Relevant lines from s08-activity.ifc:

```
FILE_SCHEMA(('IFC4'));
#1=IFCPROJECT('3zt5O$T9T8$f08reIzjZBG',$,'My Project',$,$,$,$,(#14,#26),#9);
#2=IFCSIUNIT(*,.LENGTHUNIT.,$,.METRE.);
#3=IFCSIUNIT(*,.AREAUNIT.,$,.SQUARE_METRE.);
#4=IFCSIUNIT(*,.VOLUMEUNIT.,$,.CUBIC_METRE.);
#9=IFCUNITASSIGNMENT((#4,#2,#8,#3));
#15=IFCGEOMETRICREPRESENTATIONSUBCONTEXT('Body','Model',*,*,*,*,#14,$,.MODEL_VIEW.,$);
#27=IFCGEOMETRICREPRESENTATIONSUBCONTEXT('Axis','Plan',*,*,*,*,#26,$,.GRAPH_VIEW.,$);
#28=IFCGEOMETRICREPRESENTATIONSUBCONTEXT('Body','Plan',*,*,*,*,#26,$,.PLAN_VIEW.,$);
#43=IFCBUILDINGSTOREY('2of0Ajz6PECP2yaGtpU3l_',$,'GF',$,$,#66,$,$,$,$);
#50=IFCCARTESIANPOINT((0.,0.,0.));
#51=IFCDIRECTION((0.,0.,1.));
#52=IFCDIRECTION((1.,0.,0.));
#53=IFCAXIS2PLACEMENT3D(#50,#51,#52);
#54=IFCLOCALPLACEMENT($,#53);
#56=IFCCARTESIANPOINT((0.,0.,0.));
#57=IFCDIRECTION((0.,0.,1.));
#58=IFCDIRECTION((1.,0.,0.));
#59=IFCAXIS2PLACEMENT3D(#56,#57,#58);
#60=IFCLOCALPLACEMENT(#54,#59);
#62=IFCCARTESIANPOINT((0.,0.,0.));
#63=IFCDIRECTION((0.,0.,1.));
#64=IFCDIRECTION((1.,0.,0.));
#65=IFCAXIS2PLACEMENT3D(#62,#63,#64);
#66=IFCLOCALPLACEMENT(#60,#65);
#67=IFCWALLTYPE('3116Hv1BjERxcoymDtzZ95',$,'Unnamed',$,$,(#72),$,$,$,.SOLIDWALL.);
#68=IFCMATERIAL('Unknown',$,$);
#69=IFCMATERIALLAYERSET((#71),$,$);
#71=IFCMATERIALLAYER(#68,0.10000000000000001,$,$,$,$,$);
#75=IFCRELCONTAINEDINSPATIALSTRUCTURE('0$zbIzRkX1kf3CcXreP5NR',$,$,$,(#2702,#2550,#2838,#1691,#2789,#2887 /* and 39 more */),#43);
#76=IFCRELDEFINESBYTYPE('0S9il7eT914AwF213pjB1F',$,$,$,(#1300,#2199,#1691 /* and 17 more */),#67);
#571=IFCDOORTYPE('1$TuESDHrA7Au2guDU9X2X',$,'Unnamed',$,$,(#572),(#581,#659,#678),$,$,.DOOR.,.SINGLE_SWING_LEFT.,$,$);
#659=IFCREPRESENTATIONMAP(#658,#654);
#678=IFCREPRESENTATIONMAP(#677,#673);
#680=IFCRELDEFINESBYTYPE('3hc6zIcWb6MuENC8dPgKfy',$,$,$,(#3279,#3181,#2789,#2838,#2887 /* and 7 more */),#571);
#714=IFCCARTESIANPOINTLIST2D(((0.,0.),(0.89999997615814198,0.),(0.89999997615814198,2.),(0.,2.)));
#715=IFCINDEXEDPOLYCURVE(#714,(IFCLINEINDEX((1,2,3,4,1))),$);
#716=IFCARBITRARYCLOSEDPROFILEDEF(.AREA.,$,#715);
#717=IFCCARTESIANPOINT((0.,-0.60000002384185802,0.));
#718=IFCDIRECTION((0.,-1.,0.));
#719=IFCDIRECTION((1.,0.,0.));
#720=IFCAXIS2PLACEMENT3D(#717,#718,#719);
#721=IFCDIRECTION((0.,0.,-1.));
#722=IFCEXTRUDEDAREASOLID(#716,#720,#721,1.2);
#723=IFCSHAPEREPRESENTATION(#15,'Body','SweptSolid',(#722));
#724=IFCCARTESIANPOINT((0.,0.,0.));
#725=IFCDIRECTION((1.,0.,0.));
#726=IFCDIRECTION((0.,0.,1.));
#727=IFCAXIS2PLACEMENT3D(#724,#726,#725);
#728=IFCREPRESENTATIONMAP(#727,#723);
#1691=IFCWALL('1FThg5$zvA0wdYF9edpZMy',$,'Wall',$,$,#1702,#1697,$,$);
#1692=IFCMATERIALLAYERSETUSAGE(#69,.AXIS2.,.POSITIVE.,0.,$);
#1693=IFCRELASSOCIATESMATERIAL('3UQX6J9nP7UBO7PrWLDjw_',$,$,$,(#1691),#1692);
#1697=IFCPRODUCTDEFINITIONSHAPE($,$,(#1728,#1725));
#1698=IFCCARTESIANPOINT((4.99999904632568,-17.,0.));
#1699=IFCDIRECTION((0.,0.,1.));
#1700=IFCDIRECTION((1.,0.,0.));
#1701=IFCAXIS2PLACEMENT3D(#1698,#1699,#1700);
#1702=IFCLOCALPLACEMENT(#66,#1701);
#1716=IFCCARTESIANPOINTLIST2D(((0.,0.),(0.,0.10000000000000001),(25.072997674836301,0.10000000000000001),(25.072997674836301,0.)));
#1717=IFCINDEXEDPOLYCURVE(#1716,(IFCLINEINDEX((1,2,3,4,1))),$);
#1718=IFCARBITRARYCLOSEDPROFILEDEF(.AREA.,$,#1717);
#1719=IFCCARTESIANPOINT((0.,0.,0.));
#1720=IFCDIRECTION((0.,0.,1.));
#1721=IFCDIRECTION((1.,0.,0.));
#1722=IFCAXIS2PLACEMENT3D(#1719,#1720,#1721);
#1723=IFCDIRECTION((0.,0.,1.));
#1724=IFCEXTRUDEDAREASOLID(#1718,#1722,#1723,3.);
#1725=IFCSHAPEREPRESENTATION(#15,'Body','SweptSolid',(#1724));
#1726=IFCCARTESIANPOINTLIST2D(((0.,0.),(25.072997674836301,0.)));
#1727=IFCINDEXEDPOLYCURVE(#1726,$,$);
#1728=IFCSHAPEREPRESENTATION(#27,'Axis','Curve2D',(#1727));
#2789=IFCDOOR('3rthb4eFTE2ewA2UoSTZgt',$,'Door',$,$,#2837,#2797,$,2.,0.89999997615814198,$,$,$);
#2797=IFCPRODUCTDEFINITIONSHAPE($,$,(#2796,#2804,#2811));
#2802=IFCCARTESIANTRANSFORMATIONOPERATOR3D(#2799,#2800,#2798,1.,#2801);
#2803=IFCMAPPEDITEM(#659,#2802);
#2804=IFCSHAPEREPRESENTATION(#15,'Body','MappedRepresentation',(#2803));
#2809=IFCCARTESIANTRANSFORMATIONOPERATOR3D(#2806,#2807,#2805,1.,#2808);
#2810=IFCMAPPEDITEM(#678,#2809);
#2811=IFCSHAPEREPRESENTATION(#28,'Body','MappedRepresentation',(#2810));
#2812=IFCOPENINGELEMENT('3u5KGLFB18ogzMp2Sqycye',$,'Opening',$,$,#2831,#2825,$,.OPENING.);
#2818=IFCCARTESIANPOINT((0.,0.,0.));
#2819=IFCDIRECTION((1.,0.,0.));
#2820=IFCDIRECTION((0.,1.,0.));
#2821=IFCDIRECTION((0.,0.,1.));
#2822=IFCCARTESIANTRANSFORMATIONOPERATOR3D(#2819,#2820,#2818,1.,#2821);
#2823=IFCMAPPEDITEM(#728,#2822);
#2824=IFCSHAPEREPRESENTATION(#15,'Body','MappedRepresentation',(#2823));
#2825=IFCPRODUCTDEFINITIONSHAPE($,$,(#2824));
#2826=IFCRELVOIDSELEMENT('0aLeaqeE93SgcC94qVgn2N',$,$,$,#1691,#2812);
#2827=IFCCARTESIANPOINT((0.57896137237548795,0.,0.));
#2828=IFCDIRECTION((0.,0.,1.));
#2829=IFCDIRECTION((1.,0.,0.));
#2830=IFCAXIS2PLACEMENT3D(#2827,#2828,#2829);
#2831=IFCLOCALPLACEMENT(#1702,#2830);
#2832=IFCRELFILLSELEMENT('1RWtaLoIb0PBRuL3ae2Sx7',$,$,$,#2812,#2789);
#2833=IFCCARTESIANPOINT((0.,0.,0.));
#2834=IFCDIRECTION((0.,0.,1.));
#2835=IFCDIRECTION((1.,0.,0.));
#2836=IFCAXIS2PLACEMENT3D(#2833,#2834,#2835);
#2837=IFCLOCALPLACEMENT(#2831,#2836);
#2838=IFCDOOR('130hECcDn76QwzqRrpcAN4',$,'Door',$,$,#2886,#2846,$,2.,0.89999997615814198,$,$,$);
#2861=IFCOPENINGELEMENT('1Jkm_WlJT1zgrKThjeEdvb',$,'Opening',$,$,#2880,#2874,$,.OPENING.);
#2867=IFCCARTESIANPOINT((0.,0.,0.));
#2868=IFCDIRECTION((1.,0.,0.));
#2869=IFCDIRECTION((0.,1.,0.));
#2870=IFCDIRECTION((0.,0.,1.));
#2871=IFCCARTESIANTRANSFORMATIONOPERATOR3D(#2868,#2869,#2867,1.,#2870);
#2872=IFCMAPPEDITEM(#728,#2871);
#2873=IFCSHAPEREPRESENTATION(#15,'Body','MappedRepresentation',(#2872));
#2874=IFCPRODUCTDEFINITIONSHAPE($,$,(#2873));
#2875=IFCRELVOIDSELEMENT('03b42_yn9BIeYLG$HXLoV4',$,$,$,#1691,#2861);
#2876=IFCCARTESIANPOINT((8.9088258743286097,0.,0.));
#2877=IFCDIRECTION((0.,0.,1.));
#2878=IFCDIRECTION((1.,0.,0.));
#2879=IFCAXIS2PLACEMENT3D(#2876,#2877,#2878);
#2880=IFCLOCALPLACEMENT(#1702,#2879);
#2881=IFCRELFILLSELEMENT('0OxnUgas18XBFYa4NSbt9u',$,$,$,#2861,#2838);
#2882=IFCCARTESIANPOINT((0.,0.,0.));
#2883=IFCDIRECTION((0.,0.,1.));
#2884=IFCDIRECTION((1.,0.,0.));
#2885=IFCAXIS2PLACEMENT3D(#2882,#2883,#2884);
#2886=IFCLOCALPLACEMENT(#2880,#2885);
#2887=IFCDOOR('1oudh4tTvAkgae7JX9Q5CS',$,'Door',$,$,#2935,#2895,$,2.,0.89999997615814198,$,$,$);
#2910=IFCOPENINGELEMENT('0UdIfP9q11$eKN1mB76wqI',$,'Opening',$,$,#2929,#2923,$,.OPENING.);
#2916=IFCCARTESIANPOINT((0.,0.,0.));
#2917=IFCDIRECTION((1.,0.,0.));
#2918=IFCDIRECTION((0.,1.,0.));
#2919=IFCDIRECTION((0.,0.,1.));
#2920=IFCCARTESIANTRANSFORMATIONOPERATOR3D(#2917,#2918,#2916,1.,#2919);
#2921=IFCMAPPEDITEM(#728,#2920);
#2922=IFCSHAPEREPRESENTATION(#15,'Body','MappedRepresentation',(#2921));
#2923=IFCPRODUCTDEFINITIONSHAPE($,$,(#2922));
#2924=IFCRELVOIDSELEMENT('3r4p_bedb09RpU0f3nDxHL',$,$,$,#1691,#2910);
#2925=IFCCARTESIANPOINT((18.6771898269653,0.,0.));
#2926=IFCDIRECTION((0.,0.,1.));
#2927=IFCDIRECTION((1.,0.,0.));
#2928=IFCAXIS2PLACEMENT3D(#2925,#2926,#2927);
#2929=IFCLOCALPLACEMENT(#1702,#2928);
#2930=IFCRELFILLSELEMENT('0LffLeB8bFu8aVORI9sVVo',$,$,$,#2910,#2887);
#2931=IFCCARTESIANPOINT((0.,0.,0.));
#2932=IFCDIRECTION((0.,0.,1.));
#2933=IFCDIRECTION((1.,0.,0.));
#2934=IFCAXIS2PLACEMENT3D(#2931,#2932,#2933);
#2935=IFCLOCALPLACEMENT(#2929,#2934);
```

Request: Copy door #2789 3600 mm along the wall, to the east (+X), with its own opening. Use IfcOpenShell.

```python
import ifcopenshell
import ifcopenshell.api.feature
import ifcopenshell.api.geometry
import ifcopenshell.api.root
import ifcopenshell.geom
import ifcopenshell.util.element
import ifcopenshell.util.placement
import ifcopenshell.util.shape
import ifcopenshell.util.unit

model = ifcopenshell.open("s08-activity.ifc")
unit_scale = ifcopenshell.util.unit.calculate_unit_scale(model)
settings = ifcopenshell.geom.settings()


def volume(element):
    """Net volume in cubic metres, openings subtracted."""
    shape = ifcopenshell.geom.create_shape(settings, element)
    return ifcopenshell.util.shape.get_volume(shape.geometry)


door = model.by_guid("3rthb4eFTE2ewA2UoSTZgt")
opening = door.FillsVoids[0].RelatingOpeningElement
wall = opening.VoidsElements[0].RelatingBuildingElement
before = volume(wall)
shift = ifcopenshell.util.placement.get_local_placement(wall.ObjectPlacement)[:3, 0] * 3.6 / unit_scale

# copy_class copies the void relationship, type, container and properties, but no geometry.
new_opening = ifcopenshell.api.root.copy_class(model, product=opening)
new_opening.Representation = ifcopenshell.util.element.copy_deep(
    model, opening.Representation, exclude=["IfcGeometricRepresentationContext", "IfcRepresentationMap"]
)
new_door = ifcopenshell.api.root.copy_class(model, product=door)
new_door.Representation = ifcopenshell.util.element.copy_deep(
    model, door.Representation, exclude=["IfcGeometricRepresentationContext", "IfcRepresentationMap"]
)
ifcopenshell.api.feature.add_filling(model, opening=new_opening, element=new_door)

for old, new in ((opening, new_opening), (door, new_door)):
    matrix = ifcopenshell.util.placement.get_local_placement(old.ObjectPlacement)
    matrix[:3, 3] += shift
    ifcopenshell.api.geometry.edit_object_placement(model, product=new, matrix=matrix, is_si=False)

after = volume(wall)

print(f"wall volume {before:.3f} -> {after:.3f} m3")

model.write("s08-activity_edited.ifc")
```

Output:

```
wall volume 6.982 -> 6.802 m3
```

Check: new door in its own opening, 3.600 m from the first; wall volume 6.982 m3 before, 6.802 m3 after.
